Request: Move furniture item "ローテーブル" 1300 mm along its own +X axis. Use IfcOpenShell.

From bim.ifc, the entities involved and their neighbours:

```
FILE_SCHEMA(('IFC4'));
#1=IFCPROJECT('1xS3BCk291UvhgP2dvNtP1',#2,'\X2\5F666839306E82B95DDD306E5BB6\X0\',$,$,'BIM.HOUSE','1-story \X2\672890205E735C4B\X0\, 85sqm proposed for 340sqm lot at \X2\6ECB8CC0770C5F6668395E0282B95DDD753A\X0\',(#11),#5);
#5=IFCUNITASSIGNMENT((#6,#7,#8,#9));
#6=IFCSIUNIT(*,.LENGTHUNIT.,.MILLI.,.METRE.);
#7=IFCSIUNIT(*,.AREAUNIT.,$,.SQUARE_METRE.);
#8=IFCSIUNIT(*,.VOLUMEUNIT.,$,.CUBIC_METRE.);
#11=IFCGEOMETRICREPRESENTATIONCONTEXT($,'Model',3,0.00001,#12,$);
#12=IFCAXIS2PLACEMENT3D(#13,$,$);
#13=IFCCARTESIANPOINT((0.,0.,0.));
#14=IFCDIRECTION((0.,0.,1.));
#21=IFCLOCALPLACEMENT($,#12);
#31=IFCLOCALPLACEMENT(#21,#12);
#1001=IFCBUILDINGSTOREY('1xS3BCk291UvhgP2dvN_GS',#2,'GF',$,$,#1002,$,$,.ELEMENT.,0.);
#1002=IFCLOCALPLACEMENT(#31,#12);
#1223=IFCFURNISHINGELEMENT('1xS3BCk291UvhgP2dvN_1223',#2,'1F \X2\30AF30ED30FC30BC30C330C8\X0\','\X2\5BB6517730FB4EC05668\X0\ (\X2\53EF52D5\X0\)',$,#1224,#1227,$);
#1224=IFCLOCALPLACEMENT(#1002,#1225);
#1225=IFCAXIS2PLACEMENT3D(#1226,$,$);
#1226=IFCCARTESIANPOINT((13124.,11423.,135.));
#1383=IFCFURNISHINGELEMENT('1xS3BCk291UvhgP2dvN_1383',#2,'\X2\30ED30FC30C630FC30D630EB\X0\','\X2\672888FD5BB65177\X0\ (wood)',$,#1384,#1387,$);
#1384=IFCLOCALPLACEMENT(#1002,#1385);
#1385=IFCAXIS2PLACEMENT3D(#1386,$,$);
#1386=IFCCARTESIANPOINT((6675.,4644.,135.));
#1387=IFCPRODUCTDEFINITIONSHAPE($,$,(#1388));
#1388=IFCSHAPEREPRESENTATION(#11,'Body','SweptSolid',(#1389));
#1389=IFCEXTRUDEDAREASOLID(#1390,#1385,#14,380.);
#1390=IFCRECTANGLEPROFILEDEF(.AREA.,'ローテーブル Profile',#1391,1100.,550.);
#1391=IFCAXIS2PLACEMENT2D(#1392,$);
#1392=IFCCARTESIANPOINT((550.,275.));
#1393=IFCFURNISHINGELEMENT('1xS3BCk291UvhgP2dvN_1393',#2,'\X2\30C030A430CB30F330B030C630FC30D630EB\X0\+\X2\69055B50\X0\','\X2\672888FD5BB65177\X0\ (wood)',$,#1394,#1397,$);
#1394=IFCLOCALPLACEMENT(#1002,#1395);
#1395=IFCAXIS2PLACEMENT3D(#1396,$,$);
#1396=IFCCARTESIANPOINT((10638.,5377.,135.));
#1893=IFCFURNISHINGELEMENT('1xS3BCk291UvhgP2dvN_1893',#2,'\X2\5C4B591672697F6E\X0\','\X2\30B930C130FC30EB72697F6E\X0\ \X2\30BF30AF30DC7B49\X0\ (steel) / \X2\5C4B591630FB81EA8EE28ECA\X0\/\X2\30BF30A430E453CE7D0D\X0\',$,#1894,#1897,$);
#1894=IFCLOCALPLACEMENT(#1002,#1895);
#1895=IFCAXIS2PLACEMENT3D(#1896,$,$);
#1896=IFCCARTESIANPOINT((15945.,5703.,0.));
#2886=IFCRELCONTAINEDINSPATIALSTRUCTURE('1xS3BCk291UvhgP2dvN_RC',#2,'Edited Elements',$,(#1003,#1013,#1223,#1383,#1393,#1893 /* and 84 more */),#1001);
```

```python
import ifcopenshell
import ifcopenshell.api.geometry
import ifcopenshell.util.placement
import ifcopenshell.util.unit

model = ifcopenshell.open("bim.ifc")
unit_scale = ifcopenshell.util.unit.calculate_unit_scale(model)

item = model.by_guid("1xS3BCk291UvhgP2dvN_1383")
matrix = ifcopenshell.util.placement.get_local_placement(item.ObjectPlacement)
matrix[:3, 3] += matrix[:3, 0] * 1.3 / unit_scale
ifcopenshell.api.geometry.edit_object_placement(model, product=item, matrix=matrix, is_si=False)

print(ifcopenshell.util.placement.get_local_placement(item.ObjectPlacement).round(3) + 0.0)

model.write("bim_updated.ifc")
```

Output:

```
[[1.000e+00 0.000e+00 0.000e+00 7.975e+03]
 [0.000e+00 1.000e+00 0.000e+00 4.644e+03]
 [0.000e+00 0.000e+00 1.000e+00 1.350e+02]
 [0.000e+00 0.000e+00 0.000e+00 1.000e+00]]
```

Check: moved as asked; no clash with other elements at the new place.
